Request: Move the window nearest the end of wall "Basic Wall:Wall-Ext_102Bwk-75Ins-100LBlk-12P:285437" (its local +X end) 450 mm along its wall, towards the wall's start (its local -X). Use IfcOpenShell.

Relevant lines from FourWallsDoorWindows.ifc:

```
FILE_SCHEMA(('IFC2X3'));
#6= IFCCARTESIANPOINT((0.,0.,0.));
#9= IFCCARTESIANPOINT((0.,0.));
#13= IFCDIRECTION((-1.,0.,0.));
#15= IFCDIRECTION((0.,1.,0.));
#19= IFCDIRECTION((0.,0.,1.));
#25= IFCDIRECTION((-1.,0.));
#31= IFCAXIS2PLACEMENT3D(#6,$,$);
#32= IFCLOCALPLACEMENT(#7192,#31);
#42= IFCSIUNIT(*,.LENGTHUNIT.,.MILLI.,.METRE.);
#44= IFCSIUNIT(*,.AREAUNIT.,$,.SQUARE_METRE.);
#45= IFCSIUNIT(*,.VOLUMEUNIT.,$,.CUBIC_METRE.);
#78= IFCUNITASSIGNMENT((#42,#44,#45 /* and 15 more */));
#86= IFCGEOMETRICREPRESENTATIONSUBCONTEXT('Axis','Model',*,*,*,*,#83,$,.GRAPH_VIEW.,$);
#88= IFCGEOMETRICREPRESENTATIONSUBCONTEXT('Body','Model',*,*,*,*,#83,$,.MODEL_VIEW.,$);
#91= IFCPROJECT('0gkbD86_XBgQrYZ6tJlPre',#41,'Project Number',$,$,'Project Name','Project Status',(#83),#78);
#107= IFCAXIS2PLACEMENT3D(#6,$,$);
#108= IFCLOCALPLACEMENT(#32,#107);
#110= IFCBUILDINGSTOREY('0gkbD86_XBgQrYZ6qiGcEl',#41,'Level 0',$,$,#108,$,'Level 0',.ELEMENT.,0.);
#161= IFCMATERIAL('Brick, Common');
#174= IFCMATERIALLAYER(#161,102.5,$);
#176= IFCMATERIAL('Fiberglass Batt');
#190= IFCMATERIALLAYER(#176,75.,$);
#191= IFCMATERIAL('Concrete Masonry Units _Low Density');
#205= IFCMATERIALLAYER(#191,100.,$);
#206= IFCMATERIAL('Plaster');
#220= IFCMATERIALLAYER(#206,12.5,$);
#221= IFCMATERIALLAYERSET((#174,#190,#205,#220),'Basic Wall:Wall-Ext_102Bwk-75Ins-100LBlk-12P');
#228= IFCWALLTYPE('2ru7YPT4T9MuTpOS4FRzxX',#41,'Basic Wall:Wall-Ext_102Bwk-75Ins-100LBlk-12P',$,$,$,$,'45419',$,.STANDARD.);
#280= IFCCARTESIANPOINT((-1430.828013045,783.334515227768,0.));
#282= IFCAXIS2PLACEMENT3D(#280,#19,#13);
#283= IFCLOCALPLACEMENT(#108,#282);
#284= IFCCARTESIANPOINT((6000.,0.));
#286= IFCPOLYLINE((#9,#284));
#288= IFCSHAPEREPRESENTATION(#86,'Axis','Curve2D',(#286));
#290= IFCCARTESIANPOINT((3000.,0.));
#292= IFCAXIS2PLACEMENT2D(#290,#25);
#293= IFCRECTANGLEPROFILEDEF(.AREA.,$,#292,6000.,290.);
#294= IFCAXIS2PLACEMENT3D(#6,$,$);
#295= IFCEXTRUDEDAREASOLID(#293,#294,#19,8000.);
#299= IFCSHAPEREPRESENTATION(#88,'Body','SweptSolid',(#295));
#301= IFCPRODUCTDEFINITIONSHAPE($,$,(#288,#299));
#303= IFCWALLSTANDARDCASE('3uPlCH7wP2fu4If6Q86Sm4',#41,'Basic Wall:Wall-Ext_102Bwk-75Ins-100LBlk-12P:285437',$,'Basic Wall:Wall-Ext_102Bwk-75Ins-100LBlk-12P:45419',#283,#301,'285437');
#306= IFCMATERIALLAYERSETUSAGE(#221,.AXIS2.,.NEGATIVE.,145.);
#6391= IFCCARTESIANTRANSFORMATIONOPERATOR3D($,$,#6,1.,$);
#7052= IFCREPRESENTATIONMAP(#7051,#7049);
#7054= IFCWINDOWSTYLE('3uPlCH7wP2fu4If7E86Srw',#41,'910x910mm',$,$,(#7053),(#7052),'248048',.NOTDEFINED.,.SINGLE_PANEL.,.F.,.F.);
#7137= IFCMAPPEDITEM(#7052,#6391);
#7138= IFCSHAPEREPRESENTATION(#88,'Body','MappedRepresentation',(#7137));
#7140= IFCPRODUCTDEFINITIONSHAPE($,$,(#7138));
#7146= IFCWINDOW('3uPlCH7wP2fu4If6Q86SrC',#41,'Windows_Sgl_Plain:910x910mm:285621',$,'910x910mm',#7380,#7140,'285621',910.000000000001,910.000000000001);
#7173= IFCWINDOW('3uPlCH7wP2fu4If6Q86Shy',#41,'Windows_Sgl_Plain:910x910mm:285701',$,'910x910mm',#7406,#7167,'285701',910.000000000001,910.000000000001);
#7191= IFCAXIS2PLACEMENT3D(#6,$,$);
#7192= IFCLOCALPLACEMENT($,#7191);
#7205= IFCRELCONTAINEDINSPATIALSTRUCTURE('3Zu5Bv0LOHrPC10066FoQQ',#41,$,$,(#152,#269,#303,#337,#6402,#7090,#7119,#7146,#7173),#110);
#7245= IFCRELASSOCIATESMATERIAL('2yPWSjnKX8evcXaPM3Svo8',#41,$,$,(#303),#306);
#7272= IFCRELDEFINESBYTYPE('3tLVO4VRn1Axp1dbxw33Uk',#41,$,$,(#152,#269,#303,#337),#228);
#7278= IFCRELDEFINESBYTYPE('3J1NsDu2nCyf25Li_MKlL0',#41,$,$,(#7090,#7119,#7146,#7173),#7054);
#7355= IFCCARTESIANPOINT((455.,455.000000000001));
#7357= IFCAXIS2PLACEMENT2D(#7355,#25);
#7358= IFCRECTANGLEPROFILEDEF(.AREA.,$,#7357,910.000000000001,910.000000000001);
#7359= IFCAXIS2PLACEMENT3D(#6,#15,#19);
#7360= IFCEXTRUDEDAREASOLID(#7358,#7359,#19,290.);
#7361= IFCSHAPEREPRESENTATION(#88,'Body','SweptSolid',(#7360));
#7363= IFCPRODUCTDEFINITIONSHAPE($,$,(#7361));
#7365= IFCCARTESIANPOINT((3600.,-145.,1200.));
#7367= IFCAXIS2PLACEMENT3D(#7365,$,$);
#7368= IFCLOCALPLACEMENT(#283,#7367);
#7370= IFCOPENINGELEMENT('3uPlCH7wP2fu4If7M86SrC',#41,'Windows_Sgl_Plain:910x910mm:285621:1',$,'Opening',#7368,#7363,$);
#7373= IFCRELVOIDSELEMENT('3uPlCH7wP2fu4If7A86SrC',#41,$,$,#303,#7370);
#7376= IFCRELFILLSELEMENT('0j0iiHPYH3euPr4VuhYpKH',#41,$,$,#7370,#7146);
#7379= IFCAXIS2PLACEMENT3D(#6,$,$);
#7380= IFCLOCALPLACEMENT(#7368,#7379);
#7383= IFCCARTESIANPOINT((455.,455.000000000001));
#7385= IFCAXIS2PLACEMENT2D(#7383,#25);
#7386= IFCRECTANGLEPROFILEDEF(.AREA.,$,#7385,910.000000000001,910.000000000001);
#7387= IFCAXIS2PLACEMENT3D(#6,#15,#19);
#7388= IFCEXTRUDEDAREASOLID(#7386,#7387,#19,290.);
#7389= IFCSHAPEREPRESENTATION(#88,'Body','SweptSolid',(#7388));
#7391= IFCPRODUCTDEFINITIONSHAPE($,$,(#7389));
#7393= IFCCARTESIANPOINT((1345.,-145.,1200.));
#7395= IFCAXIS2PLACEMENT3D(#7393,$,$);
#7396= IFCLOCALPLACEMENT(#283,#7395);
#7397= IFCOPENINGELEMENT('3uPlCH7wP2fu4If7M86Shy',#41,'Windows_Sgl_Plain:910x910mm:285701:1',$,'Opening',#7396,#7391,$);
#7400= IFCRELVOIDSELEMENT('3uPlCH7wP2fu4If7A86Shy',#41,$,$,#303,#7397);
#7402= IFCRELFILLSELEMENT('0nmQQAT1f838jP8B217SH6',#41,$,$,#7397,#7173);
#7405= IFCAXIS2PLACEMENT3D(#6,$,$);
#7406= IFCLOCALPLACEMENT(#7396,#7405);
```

```python
import ifcopenshell
import ifcopenshell.api.geometry
import ifcopenshell.util.placement
import ifcopenshell.util.unit

model = ifcopenshell.open("FourWallsDoorWindows.ifc")
unit_scale = ifcopenshell.util.unit.calculate_unit_scale(model)

window = model.by_guid("3uPlCH7wP2fu4If6Q86SrC")
opening = window.FillsVoids[0].RelatingOpeningElement
wall = opening.VoidsElements[0].RelatingBuildingElement

wall_matrix = ifcopenshell.util.placement.get_local_placement(wall.ObjectPlacement)
shift = wall_matrix[:3, 0] * -0.45 / unit_scale
before = ifcopenshell.util.placement.get_local_placement(window.ObjectPlacement)[:3, 3].copy()

# The window is placed relative to its opening, so it follows when the opening moves.
matrix = ifcopenshell.util.placement.get_local_placement(opening.ObjectPlacement)
matrix[:3, 3] += shift
ifcopenshell.api.geometry.edit_object_placement(
    model, product=opening, matrix=matrix, is_si=False, should_transform_children=True
)

after = ifcopenshell.util.placement.get_local_placement(window.ObjectPlacement)[:3, 3]
print("window moved by", (after - before).round(3) + 0.0)

model.write("FourWallsDoorWindows_edited.ifc")
```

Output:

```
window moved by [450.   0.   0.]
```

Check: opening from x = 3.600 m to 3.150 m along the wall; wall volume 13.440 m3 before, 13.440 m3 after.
